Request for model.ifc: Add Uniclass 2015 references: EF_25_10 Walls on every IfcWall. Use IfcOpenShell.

First a look at what the model holds.

```python
import ifcopenshell

model = ifcopenshell.open("model.ifc")
print(model.schema)
print("classifications:", [c.Name for c in model.by_type("IfcClassification")])
for ifc_class in ("IfcDoor", "IfcRoof", "IfcStair", "IfcWall", "IfcWindow"):
    print(ifc_class, len(model.by_type(ifc_class)))
```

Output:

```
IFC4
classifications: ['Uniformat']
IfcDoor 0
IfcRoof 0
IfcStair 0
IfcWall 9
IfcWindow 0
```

```python
import ifcopenshell
import ifcopenshell.api.classification

model = ifcopenshell.open("model.ifc")

system = ifcopenshell.api.classification.add_classification(model, classification="Uniclass 2015")

codes = {
    "IfcWall": ("EF_25_10", "Walls"),
}
for ifc_class, (code, name) in codes.items():
    products = model.by_type(ifc_class)
    ifcopenshell.api.classification.add_reference(
        model, products=products, classification=system, identification=code, name=name
    )
    print(code, len(products))

model.write("model_edited.ifc")
```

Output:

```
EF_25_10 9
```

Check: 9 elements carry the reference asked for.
